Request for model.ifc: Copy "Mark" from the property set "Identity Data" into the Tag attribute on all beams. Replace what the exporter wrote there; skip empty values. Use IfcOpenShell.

First a look at what the model holds.

```python
import ifcopenshell
import ifcopenshell.util.element

model = ifcopenshell.open("model.ifc")
print(model.schema)
beams = model.by_type("IfcBeam")
print(len(beams), "beams")
for e in beams[:8]:
    source = ifcopenshell.util.element.get_pset(e, "Identity Data", "Mark")
    target = e.Tag
    print(e.id(), repr(source), repr(target), sep=" | ")
```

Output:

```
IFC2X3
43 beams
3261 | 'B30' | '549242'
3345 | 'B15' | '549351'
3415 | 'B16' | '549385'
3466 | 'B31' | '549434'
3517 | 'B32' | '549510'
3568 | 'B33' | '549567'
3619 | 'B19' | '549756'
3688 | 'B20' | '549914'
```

```python
import ifcopenshell
import ifcopenshell.util.element

model = ifcopenshell.open("model.ifc")

count = 0
for e in model.by_type("IfcBeam"):
    value = ifcopenshell.util.element.get_pset(e, "Identity Data", "Mark")
    current = e.Tag
    if not value or not value.strip() or current == value:
        continue
    e.Tag = value
    count += 1

print(count, "beams updated")

model.write("model_updated.ifc")
```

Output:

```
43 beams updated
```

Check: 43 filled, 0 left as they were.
